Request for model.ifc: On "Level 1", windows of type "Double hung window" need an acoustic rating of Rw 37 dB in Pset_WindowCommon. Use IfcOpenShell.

First a look at what the model holds.

```python
import ifcopenshell
import ifcopenshell.util.element

model = ifcopenshell.open("model.ifc")
print(model.schema)
storey = next(s for s in model.by_type("IfcBuildingStorey") if s.Name == "Level 1")
windows = [e for e in ifcopenshell.util.element.get_decomposition(storey) if e.is_a("IfcWindow")]
seen = {}
for e in windows:
    element_type = ifcopenshell.util.element.get_type(e)
    key = (element_type.Name if element_type != e and element_type else None, ifcopenshell.util.element.get_pset(e, "Pset_WindowCommon", "AcousticRating"))
    seen[key] = seen.get(key, 0) + 1
for (name, value), count in sorted(seen.items(), key=str):
    print(count, "x", name, "|", value)
```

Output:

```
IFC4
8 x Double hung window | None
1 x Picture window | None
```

```python
import ifcopenshell
import ifcopenshell.api.pset
import ifcopenshell.util.element

model = ifcopenshell.open("model.ifc")

storey = next(s for s in model.by_type("IfcBuildingStorey") if s.Name == "Level 1")
windows = [e for e in ifcopenshell.util.element.get_decomposition(storey) if e.is_a("IfcWindow")]

count = 0
for e in windows:
    element_type = ifcopenshell.util.element.get_type(e)
    if element_type in (None, e) or element_type.Name != "Double hung window":
        continue
    # add_pset returns the element's existing set when there is one.
    pset = ifcopenshell.api.pset.add_pset(model, product=e, name="Pset_WindowCommon")
    ifcopenshell.api.pset.edit_pset(model, pset=pset, properties={"AcousticRating": "Rw 37 dB"})
    count += 1

print(count, "windows updated")

model.write("model_edited.ifc")
```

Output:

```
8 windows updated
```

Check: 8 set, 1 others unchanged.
